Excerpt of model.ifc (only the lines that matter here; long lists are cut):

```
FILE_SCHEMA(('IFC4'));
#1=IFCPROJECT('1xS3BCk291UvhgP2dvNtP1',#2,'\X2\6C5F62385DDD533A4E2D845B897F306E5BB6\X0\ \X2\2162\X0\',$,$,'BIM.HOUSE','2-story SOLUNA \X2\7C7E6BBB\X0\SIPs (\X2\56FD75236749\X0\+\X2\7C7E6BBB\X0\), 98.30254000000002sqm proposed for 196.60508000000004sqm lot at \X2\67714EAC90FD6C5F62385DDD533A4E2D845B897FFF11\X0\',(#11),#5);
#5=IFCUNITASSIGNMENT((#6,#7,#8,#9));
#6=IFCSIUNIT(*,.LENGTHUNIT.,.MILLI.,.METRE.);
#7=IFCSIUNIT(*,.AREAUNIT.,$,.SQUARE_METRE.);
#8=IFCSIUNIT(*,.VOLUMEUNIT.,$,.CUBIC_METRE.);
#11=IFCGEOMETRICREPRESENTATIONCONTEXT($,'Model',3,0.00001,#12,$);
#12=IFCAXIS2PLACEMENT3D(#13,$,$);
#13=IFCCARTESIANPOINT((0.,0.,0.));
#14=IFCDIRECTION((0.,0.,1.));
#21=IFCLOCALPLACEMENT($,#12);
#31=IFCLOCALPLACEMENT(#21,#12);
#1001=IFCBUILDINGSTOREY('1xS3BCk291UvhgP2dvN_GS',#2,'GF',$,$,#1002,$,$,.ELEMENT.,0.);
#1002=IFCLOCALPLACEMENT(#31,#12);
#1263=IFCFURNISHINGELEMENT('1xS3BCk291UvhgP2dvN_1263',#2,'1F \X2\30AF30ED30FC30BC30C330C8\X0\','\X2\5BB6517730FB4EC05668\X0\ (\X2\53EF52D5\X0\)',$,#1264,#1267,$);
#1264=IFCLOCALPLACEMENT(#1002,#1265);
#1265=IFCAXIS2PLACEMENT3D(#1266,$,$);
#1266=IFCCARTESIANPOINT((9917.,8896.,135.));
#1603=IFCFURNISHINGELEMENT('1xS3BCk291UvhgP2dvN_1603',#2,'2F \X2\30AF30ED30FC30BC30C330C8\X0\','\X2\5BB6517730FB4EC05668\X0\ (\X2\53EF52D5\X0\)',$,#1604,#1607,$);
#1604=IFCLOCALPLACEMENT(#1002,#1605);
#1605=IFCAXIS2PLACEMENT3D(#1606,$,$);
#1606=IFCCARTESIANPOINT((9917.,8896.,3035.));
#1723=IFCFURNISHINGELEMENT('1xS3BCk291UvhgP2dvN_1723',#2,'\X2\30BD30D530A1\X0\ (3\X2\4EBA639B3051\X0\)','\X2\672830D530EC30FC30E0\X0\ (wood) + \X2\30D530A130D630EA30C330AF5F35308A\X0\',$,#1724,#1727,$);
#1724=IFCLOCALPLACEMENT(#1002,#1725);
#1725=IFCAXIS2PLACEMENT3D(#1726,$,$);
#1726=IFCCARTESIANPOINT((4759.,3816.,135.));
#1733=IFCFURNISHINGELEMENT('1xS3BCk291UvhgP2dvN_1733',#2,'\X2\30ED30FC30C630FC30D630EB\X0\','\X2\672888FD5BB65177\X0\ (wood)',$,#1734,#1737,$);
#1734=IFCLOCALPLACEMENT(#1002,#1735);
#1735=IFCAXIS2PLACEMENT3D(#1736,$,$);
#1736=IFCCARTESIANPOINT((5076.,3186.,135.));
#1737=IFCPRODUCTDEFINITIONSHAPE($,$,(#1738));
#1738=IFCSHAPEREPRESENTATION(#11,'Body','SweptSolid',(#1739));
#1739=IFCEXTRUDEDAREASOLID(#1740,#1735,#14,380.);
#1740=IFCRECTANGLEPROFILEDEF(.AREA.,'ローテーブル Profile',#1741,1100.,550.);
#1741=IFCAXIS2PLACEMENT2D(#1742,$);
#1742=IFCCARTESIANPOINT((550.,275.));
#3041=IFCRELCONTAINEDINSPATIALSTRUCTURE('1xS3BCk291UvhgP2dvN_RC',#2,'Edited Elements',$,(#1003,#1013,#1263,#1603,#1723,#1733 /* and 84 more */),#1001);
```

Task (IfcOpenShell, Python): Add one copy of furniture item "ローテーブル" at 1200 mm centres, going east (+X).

```python
import numpy as np
import ifcopenshell
import ifcopenshell.api.geometry
import ifcopenshell.api.root
import ifcopenshell.util.element
import ifcopenshell.util.placement

model = ifcopenshell.open("model.ifc")


def reuse_history(source, copy):
    """copy_class also copies each property set's owner history, people and application; keep the originals."""
    for rel in copy.IsDefinedBy:
        if rel.is_a("IfcRelDefinesByProperties") and (history := rel.RelatingPropertyDefinition.OwnerHistory):
            rel.RelatingPropertyDefinition.OwnerHistory = source.OwnerHistory
            ifcopenshell.util.element.remove_deep2(model, history)


source = model.by_guid("1xS3BCk291UvhgP2dvN_1733")
base = ifcopenshell.util.placement.get_local_placement(source.ObjectPlacement)
step = np.array([1.0, 0.0, 0.0]) * 1200.0

for i in range(1, 2):
    copy = ifcopenshell.api.root.copy_class(model, product=source)
    copy.Representation = ifcopenshell.util.element.copy_deep(
        model, source.Representation, exclude=["IfcGeometricRepresentationContext", "IfcRepresentationMap"]
    )
    reuse_history(source, copy)
    matrix = base.copy()
    matrix[:3, 3] += i * step
    print("added at", matrix[:3, 3].round(3) + 0.0)
    ifcopenshell.api.geometry.edit_object_placement(model, product=copy, matrix=matrix, is_si=False)

model.write("model_updated.ifc")
```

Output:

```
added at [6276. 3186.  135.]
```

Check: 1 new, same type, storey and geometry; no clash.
